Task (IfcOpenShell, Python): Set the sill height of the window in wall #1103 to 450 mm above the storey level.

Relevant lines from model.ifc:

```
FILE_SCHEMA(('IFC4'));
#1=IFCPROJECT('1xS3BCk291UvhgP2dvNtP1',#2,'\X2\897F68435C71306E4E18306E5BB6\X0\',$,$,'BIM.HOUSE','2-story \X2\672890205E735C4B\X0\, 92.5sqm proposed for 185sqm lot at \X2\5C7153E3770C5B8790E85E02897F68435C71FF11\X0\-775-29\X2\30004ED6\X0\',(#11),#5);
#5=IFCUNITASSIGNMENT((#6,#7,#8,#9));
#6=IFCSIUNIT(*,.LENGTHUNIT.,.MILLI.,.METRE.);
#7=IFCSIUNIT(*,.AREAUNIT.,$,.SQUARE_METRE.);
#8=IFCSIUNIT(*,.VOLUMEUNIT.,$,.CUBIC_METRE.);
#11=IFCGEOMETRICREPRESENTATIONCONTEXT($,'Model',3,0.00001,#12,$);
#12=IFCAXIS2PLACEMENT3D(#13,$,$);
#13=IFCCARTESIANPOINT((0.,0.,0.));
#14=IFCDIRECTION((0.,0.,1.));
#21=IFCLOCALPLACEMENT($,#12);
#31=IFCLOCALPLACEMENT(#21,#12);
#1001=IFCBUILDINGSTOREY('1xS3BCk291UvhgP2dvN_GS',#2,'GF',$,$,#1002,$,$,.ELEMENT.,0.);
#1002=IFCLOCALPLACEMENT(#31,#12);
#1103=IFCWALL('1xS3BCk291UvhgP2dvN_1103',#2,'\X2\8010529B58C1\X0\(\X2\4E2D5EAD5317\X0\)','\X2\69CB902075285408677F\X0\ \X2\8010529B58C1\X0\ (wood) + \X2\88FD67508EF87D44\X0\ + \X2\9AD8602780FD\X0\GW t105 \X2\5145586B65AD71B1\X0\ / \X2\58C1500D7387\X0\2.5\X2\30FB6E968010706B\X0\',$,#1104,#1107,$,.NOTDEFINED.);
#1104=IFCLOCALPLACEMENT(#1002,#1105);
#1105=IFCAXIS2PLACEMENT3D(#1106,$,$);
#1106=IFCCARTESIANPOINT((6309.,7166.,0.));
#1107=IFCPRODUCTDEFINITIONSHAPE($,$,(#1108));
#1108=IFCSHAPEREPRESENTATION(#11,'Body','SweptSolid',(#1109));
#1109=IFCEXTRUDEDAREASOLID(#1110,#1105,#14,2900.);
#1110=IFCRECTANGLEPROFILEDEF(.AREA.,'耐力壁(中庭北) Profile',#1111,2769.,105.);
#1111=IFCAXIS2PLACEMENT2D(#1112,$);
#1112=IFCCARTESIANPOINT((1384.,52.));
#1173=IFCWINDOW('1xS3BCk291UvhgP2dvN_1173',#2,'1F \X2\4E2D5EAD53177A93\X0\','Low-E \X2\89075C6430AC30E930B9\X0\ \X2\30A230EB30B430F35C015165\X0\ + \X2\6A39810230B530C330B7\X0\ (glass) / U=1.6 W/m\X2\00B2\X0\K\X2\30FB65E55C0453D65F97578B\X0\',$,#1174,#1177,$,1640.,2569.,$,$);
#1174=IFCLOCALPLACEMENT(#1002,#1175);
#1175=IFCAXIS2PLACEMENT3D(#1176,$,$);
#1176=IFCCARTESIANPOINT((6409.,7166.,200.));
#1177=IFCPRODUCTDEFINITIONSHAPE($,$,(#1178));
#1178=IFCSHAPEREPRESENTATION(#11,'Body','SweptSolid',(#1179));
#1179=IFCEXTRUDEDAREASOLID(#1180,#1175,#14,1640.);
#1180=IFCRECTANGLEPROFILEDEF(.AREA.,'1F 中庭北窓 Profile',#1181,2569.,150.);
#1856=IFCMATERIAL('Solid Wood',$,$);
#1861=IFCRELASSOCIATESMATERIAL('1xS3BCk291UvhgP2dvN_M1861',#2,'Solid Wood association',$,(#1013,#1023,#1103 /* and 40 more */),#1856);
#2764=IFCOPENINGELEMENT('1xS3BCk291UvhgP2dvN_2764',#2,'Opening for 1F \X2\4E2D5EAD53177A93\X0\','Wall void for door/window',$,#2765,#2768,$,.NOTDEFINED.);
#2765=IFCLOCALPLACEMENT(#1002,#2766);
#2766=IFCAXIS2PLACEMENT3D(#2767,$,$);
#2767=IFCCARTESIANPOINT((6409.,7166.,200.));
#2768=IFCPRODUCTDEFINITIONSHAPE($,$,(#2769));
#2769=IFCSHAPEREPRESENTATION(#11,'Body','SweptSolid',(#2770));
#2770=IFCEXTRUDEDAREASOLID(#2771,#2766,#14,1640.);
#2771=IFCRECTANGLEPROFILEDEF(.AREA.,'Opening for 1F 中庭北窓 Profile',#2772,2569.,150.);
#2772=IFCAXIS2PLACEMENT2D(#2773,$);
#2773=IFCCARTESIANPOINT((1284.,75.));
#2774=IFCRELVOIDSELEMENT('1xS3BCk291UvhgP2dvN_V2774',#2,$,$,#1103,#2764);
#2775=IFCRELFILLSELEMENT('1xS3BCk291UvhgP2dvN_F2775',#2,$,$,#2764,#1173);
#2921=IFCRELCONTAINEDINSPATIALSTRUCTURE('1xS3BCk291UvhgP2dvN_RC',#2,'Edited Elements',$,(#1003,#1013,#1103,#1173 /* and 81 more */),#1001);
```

```python
import numpy as np
import ifcopenshell
import ifcopenshell.api.geometry
import ifcopenshell.geom
import ifcopenshell.util.element
import ifcopenshell.util.placement
import ifcopenshell.util.shape
import ifcopenshell.util.unit

model = ifcopenshell.open("model.ifc")
unit_scale = ifcopenshell.util.unit.calculate_unit_scale(model)

window = model.by_guid("1xS3BCk291UvhgP2dvN_1173")
opening = window.FillsVoids[0].RelatingOpeningElement
storey = ifcopenshell.util.element.get_container(window, ifc_class="IfcBuildingStorey")
level = ifcopenshell.util.placement.get_local_placement(storey.ObjectPlacement)[2, 3]

# The opening's origin need not be at the sill, so measure its lowest point.
shape = ifcopenshell.geom.create_shape(ifcopenshell.geom.settings(), opening)
bottom = ifcopenshell.util.shape.get_shape_bottom_elevation(shape, shape.geometry) / unit_scale
dz = level + 0.45 / unit_scale - bottom

shift = np.array([0.0, 0.0, dz])
# The window is not placed relative to its opening, so move both.
for product in (opening, window):
    matrix = ifcopenshell.util.placement.get_local_placement(product.ObjectPlacement)
    matrix[:3, 3] += shift
    ifcopenshell.api.geometry.edit_object_placement(model, product=product, matrix=matrix, is_si=False)

print(f"moved by {dz * unit_scale:+.3f} m")

model.write("model_v2.ifc")
```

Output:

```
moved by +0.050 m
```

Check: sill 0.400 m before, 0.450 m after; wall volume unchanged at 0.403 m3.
